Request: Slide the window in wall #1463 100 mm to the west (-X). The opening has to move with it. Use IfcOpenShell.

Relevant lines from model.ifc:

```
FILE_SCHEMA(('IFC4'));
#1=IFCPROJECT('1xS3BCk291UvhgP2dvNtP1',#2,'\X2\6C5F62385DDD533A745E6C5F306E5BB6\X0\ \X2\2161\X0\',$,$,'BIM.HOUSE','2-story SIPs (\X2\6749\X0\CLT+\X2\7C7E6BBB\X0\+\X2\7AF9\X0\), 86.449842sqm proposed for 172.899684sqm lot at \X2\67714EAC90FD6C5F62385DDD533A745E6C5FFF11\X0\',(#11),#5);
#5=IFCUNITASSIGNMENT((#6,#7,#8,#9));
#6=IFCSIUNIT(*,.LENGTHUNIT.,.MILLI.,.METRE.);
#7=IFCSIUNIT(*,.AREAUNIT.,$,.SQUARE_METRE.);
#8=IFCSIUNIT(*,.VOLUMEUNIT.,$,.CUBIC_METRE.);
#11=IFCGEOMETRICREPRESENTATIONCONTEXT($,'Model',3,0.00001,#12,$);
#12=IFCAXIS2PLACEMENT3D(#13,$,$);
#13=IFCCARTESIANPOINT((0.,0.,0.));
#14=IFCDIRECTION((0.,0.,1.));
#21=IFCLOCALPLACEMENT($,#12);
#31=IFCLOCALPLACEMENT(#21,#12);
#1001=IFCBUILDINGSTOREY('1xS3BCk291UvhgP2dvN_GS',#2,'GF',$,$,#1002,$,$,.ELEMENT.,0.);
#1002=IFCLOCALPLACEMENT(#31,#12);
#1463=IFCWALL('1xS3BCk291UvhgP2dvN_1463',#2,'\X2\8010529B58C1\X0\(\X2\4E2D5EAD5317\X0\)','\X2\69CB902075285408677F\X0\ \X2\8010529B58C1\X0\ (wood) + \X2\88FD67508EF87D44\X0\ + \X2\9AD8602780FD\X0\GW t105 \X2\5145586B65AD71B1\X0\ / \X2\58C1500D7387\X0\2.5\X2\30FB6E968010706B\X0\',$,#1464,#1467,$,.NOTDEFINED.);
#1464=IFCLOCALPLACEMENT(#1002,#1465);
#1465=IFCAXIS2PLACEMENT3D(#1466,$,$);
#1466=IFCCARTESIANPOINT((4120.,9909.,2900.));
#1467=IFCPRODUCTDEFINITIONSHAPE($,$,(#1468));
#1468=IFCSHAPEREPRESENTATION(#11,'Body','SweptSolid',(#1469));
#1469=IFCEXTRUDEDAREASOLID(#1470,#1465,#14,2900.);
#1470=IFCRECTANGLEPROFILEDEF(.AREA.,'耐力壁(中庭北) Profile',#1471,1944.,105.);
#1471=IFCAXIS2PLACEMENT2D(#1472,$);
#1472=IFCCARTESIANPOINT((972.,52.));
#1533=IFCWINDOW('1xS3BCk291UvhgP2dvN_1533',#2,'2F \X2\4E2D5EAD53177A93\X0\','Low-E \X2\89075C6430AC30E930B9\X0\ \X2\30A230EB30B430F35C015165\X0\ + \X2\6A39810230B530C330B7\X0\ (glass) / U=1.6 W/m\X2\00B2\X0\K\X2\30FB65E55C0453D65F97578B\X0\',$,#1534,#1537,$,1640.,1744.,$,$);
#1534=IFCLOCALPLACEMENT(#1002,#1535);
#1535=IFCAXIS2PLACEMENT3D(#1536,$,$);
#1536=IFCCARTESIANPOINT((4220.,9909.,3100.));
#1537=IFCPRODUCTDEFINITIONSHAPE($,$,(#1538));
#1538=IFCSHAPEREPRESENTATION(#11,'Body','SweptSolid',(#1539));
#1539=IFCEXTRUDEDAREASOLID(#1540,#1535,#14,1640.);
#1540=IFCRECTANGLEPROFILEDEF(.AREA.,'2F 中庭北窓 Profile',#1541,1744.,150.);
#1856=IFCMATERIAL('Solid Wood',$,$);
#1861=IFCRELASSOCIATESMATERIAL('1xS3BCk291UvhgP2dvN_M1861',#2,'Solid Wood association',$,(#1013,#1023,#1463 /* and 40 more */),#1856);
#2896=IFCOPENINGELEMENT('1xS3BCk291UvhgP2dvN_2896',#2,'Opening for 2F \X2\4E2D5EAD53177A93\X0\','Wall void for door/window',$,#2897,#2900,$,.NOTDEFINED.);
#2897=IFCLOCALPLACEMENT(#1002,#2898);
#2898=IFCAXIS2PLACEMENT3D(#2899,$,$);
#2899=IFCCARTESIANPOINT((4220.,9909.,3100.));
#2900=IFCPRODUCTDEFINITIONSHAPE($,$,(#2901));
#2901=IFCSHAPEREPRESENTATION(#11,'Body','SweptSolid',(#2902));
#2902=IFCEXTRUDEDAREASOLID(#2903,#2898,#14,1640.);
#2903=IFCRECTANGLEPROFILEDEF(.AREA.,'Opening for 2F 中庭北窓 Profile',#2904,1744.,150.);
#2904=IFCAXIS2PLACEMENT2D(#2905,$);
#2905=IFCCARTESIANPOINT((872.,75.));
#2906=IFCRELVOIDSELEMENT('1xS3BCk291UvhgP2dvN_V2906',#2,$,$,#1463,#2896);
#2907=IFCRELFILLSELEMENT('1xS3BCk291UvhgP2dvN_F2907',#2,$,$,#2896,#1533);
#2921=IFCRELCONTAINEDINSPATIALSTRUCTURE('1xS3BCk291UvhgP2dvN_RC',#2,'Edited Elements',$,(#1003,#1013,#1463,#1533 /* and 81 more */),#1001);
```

```python
import ifcopenshell
import ifcopenshell.api.geometry
import ifcopenshell.util.placement
import ifcopenshell.util.unit

model = ifcopenshell.open("model.ifc")
unit_scale = ifcopenshell.util.unit.calculate_unit_scale(model)

window = model.by_id(1533)
opening = window.FillsVoids[0].RelatingOpeningElement
wall = opening.VoidsElements[0].RelatingBuildingElement

wall_matrix = ifcopenshell.util.placement.get_local_placement(wall.ObjectPlacement)
shift = wall_matrix[:3, 0] * -0.1 / unit_scale
before = ifcopenshell.util.placement.get_local_placement(window.ObjectPlacement)[:3, 3].copy()

# The window is not placed relative to its opening, so move both.
for product in (opening, window):
    matrix = ifcopenshell.util.placement.get_local_placement(product.ObjectPlacement)
    matrix[:3, 3] += shift
    ifcopenshell.api.geometry.edit_object_placement(model, product=product, matrix=matrix, is_si=False)

after = ifcopenshell.util.placement.get_local_placement(window.ObjectPlacement)[:3, 3]
print("window moved by", (after - before).round(3) + 0.0)

model.write("model_edited.ifc")
```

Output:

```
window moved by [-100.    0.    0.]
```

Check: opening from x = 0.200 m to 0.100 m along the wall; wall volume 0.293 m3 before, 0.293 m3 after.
